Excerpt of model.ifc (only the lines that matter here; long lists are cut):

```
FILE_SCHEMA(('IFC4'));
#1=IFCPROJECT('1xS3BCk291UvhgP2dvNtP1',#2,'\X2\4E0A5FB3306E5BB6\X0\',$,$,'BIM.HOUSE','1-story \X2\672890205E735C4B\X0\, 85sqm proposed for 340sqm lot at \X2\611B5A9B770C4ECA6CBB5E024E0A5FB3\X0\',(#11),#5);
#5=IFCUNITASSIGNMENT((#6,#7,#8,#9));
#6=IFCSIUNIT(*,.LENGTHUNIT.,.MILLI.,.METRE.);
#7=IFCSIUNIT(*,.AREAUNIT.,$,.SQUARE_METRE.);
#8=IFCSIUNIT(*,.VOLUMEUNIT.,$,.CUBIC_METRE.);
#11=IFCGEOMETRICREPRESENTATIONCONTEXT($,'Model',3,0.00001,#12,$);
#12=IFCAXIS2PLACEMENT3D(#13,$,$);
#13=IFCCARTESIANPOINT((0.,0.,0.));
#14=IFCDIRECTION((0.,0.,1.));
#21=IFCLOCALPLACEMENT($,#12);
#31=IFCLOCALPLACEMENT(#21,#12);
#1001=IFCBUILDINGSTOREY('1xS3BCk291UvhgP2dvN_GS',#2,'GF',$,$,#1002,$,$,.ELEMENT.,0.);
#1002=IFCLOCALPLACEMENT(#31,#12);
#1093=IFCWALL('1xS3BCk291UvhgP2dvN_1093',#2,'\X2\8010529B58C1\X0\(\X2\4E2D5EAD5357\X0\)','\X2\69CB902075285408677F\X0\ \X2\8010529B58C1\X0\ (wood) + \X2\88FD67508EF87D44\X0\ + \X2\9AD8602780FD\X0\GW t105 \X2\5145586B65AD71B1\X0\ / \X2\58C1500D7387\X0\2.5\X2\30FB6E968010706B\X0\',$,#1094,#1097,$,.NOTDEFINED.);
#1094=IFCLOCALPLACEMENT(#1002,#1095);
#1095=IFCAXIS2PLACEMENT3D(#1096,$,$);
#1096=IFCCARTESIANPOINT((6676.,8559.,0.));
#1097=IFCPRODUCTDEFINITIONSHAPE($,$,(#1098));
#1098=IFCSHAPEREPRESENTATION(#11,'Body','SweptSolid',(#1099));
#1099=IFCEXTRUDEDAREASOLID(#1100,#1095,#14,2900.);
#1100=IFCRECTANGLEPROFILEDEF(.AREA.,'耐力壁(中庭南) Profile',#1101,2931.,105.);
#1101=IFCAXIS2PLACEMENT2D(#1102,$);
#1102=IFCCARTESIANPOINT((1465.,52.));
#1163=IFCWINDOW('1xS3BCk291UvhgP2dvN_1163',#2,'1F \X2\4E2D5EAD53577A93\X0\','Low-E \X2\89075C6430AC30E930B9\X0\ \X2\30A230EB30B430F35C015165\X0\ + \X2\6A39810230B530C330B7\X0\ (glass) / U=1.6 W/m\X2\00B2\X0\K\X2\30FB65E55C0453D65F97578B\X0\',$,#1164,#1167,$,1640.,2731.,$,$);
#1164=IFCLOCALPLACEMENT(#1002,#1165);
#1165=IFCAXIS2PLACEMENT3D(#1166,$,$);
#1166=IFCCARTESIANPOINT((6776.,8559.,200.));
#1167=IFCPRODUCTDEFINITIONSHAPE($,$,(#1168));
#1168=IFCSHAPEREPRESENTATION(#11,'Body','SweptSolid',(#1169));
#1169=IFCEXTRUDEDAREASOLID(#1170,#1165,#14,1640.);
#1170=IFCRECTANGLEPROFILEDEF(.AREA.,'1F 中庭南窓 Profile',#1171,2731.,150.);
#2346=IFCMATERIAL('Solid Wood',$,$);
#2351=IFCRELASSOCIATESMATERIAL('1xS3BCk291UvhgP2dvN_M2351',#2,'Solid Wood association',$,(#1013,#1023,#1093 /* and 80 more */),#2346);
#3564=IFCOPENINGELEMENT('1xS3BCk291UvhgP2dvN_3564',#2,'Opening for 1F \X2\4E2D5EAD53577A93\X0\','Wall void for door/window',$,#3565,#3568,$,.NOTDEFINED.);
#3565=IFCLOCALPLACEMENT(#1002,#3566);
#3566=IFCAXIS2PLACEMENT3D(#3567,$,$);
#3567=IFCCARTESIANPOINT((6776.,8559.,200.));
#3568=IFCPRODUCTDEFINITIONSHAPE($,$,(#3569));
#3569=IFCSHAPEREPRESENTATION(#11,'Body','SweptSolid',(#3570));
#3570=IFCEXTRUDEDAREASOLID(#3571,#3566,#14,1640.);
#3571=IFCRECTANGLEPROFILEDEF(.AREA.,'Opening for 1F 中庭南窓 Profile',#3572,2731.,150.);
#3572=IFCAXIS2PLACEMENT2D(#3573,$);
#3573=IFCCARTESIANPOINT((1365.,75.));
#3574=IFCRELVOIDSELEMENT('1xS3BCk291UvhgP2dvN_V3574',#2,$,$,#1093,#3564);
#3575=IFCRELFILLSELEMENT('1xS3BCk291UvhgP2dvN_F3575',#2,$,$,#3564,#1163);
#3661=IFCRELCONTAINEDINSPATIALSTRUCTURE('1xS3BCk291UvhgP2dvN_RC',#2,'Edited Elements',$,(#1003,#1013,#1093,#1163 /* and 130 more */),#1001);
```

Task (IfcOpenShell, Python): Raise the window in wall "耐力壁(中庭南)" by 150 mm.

```python
import numpy as np
import ifcopenshell
import ifcopenshell.api.geometry
import ifcopenshell.util.placement
import ifcopenshell.util.unit

model = ifcopenshell.open("model.ifc")
unit_scale = ifcopenshell.util.unit.calculate_unit_scale(model)

window = model.by_id(1163)
opening = window.FillsVoids[0].RelatingOpeningElement
dz = 150.0

shift = np.array([0.0, 0.0, dz])
# The window is not placed relative to its opening, so move both.
for product in (opening, window):
    matrix = ifcopenshell.util.placement.get_local_placement(product.ObjectPlacement)
    matrix[:3, 3] += shift
    ifcopenshell.api.geometry.edit_object_placement(model, product=product, matrix=matrix, is_si=False)

print(f"moved by {dz * unit_scale:+.3f} m")

model.write("model-out.ifc")
```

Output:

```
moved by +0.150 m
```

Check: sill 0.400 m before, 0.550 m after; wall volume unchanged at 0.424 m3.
